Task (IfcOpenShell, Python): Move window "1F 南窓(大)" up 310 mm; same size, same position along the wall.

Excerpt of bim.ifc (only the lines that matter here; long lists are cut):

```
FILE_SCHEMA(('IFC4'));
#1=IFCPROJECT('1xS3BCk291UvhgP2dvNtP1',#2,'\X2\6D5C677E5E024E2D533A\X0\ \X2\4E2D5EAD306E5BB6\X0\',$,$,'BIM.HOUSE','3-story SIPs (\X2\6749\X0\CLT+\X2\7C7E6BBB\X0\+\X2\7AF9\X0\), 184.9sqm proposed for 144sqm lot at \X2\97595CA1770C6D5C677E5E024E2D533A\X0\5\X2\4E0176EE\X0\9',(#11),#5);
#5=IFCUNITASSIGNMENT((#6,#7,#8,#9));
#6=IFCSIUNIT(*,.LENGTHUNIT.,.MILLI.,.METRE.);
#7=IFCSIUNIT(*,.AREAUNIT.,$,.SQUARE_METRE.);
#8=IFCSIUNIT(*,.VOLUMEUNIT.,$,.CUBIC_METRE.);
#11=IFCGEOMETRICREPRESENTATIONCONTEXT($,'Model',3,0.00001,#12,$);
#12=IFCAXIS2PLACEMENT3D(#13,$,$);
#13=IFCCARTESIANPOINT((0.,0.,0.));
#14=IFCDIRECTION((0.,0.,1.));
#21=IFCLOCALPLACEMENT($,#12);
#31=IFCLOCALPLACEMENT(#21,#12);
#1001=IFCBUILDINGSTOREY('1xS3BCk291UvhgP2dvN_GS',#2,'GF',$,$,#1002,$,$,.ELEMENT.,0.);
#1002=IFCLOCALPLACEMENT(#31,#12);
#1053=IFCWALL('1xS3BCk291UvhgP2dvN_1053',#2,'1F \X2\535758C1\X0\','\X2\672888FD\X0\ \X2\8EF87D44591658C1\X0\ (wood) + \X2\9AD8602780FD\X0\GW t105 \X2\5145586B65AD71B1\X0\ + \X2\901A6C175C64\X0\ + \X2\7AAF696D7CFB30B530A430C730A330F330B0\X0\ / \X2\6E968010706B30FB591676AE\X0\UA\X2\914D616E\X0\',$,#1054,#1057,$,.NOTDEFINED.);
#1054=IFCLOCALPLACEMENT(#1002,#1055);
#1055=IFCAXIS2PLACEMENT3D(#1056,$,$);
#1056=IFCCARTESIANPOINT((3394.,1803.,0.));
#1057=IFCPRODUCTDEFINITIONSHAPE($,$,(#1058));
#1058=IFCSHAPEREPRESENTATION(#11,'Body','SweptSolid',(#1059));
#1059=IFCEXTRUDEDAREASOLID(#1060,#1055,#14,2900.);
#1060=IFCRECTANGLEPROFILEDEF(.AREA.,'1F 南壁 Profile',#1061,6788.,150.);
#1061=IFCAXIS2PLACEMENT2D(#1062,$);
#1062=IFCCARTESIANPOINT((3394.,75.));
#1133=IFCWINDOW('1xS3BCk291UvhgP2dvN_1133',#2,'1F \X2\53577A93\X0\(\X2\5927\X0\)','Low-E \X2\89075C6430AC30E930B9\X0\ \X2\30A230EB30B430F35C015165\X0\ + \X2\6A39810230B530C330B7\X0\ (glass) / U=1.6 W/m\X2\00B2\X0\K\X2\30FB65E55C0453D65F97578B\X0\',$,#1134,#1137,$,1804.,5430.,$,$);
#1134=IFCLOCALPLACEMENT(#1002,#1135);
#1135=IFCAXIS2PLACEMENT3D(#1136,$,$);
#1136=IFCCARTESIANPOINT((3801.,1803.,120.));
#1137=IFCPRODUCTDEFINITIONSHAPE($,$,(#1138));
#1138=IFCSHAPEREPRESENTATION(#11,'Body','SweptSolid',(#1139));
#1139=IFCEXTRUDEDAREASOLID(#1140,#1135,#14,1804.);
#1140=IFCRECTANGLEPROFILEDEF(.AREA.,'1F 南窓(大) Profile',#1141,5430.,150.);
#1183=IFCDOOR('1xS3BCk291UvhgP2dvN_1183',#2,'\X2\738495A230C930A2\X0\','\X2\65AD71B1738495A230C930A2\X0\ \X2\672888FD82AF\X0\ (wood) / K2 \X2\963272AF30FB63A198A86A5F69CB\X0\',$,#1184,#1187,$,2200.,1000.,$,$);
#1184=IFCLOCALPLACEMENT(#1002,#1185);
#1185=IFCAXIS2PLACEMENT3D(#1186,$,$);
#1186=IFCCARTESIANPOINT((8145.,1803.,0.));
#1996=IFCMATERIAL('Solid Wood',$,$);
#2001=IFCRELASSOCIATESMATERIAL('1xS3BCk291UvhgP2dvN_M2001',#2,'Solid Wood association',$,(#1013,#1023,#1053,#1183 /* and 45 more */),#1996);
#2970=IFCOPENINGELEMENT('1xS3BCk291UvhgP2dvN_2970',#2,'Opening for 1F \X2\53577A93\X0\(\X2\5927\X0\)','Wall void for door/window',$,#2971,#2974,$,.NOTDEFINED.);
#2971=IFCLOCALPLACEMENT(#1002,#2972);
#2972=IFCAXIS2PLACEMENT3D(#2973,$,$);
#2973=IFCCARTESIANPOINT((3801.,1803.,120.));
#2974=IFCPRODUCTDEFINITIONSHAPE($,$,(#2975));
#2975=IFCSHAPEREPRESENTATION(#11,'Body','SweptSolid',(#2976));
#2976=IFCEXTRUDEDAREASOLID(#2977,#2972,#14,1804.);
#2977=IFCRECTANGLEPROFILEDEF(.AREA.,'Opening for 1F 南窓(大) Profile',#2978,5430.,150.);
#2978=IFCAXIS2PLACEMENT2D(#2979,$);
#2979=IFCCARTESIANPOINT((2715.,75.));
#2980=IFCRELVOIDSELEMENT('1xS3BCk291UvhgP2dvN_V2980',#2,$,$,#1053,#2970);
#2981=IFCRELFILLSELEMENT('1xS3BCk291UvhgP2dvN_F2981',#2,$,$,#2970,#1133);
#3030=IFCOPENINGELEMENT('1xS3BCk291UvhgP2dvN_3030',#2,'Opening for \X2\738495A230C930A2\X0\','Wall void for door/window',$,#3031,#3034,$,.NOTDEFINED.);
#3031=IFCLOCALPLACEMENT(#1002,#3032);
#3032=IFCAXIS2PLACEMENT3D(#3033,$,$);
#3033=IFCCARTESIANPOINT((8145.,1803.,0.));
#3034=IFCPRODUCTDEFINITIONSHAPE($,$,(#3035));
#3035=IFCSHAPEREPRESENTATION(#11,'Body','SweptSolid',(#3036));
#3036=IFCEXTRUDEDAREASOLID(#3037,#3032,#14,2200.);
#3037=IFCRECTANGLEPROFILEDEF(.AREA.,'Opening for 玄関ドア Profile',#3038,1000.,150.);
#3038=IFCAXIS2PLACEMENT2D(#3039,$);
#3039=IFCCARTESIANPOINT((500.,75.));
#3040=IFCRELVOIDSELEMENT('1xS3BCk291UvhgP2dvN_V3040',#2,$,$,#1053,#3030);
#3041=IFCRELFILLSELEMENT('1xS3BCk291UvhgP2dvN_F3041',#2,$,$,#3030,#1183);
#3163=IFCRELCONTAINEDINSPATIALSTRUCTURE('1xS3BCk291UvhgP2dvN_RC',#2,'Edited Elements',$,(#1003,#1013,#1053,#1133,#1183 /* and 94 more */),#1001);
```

```python
import numpy as np
import ifcopenshell
import ifcopenshell.api.geometry
import ifcopenshell.util.placement
import ifcopenshell.util.unit

model = ifcopenshell.open("bim.ifc")
unit_scale = ifcopenshell.util.unit.calculate_unit_scale(model)

window = model.by_guid("1xS3BCk291UvhgP2dvN_1133")
opening = window.FillsVoids[0].RelatingOpeningElement
dz = 0.31 / unit_scale

shift = np.array([0.0, 0.0, dz])
# The window is not placed relative to its opening, so move both.
for product in (opening, window):
    matrix = ifcopenshell.util.placement.get_local_placement(product.ObjectPlacement)
    matrix[:3, 3] += shift
    ifcopenshell.api.geometry.edit_object_placement(model, product=product, matrix=matrix, is_si=False)

print(f"moved by {dz * unit_scale:+.3f} m")

model.write("bim_v2.ifc")
```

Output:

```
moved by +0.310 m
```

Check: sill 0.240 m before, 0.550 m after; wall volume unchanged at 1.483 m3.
